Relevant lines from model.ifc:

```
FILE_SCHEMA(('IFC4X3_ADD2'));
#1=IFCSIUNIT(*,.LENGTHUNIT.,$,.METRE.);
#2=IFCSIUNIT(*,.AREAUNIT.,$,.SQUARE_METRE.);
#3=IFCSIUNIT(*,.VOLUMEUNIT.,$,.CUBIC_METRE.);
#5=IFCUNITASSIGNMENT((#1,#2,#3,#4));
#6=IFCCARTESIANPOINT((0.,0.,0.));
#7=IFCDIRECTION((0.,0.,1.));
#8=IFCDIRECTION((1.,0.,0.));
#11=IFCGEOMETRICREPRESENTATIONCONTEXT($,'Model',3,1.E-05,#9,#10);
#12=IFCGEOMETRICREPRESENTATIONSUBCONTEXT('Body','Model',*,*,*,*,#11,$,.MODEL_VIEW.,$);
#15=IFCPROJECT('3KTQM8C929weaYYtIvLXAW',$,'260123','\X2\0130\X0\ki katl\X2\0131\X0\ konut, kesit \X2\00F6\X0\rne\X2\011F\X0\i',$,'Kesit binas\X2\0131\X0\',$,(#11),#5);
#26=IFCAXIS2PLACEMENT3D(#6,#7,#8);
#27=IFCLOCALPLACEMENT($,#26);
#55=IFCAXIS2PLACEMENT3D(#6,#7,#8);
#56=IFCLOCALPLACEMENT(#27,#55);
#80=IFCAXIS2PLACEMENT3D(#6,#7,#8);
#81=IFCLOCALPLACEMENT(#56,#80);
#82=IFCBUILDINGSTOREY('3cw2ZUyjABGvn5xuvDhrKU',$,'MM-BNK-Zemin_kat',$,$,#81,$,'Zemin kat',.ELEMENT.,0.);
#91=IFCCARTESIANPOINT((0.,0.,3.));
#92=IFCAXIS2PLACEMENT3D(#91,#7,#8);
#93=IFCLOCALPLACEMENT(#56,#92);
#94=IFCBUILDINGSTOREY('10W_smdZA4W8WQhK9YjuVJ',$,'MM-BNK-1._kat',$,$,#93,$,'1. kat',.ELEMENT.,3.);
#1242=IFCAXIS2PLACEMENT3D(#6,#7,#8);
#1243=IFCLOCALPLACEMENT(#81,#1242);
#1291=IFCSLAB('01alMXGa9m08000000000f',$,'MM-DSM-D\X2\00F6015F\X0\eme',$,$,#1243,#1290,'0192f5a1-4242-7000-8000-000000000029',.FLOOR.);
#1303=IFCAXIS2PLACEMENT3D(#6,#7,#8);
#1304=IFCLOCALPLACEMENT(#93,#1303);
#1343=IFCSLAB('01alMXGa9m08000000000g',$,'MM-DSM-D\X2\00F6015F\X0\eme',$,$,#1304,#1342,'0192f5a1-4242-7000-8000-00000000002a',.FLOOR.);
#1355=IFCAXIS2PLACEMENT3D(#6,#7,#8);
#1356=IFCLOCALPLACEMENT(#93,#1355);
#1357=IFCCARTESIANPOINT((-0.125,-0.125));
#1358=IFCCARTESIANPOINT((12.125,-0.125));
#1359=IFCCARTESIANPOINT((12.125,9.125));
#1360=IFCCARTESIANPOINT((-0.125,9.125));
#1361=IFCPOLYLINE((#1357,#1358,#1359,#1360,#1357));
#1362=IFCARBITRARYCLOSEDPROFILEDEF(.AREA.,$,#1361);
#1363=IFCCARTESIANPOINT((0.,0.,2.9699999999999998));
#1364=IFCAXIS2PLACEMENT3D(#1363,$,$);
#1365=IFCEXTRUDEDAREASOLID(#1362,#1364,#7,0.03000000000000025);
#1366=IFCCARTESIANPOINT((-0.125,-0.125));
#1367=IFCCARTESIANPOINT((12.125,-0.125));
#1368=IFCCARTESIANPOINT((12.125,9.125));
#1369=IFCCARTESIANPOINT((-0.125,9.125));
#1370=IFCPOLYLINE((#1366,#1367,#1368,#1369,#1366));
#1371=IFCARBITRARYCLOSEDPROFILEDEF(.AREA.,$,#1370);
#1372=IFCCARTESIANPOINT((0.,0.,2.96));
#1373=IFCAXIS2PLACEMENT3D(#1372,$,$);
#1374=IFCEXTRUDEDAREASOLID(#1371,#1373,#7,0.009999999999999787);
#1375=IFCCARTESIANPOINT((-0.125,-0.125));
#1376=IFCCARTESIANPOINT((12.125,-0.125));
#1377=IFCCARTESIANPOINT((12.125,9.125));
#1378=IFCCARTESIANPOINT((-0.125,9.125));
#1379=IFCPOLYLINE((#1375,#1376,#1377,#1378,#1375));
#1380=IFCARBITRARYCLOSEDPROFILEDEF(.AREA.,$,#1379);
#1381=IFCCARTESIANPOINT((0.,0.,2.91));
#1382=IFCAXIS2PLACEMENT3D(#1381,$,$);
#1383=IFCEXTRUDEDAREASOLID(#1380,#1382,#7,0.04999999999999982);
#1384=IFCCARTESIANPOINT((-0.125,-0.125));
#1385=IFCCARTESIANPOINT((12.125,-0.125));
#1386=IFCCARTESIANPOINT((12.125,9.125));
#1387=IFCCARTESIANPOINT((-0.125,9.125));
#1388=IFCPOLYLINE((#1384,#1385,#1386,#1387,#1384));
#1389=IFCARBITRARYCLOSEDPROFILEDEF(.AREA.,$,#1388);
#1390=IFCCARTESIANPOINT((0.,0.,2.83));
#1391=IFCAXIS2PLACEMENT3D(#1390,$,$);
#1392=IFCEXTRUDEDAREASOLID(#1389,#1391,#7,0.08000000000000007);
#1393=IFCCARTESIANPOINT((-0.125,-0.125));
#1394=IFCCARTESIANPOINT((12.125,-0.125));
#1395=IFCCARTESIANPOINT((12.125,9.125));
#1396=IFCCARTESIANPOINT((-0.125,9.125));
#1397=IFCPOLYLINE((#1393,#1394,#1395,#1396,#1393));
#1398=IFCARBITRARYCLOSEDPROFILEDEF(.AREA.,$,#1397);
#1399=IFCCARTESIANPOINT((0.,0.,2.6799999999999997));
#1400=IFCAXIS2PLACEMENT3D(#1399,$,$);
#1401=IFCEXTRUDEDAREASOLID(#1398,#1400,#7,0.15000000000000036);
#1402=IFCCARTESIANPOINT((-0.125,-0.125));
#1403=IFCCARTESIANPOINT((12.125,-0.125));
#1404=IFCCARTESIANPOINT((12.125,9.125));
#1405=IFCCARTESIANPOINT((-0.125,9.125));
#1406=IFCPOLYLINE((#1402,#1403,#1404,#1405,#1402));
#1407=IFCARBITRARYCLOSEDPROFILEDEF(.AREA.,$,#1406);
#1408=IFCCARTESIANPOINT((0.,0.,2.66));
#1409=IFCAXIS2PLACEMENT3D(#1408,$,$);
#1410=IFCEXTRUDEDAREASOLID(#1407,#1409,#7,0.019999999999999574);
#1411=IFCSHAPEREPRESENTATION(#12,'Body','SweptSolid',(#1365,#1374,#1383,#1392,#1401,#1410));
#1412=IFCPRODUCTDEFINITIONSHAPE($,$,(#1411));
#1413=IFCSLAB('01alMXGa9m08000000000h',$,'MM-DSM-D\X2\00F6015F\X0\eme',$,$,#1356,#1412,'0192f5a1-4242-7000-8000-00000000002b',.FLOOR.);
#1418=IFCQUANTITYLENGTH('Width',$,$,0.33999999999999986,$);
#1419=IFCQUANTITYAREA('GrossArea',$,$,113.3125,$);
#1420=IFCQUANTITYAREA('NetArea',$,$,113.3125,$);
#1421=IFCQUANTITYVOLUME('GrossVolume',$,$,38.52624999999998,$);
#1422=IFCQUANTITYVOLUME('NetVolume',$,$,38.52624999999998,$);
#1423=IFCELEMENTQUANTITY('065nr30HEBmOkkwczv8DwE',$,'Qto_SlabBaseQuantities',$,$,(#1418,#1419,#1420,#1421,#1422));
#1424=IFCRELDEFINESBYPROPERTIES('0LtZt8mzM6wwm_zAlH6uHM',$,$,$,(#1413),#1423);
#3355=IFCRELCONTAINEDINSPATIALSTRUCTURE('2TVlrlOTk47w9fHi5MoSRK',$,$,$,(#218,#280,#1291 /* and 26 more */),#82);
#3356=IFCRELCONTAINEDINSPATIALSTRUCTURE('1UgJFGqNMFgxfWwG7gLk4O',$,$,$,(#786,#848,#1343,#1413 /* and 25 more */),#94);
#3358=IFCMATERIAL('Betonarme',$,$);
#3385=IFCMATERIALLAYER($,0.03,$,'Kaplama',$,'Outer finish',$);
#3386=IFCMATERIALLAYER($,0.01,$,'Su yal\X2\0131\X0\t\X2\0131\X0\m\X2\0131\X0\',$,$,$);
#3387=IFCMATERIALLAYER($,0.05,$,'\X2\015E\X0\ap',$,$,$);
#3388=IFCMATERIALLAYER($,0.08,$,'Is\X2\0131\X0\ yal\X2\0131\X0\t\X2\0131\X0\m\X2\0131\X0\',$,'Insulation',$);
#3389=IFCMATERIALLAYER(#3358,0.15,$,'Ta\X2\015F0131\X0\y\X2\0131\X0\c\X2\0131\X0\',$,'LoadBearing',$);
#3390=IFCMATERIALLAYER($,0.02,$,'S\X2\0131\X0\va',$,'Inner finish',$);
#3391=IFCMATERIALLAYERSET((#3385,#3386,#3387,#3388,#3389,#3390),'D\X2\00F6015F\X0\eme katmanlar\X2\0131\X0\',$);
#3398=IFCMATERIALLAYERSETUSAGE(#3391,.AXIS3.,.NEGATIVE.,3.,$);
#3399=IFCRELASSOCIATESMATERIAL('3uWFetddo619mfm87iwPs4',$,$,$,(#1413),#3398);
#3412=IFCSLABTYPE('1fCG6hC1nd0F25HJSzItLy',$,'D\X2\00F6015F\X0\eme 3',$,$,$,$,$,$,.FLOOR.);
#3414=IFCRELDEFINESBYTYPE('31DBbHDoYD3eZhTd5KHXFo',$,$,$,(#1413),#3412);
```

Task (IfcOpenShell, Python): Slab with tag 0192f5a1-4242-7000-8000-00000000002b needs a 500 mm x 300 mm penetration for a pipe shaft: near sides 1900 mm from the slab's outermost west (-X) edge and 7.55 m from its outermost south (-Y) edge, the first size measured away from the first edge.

```python
import numpy as np
import ifcopenshell
import ifcopenshell.api.feature
import ifcopenshell.api.geometry
import ifcopenshell.api.pset
import ifcopenshell.api.root
import ifcopenshell.geom
import ifcopenshell.util.element
import ifcopenshell.util.placement
import ifcopenshell.util.representation
import ifcopenshell.util.shape
import ifcopenshell.util.unit

model = ifcopenshell.open("model.ifc")
unit_scale = ifcopenshell.util.unit.calculate_unit_scale(model)
area_scale = ifcopenshell.util.unit.calculate_unit_scale(model, "AREAUNIT")
volume_scale = ifcopenshell.util.unit.calculate_unit_scale(model, "VOLUMEUNIT")
settings = ifcopenshell.geom.settings()


def volume(element):
    """Net volume in cubic metres, openings subtracted."""
    shape = ifcopenshell.geom.create_shape(settings, element)
    return ifcopenshell.util.shape.get_volume(shape.geometry)


slab = model.by_id(1413)
before = volume(slab)

# Extent in the slab's own axes, in metres. The edges named are its -X and -Y sides.
slab_shape = ifcopenshell.geom.create_shape(settings, slab)
vertices = ifcopenshell.util.shape.get_vertices(slab_shape.geometry)
x_min, y_min, bottom = vertices.min(axis=0)
top = vertices[:, 2].max()

opening = ifcopenshell.api.root.create_entity(model, ifc_class="IfcOpeningElement", name="Pipe shaft opening", predefined_type="OPENING")
context = ifcopenshell.util.representation.get_context(model, "Model", "Body", "MODEL_VIEW")
width, depth = 0.5, 0.3
outline = [(0.0, 0.0), (width, 0.0), (width, depth), (0.0, depth), (0.0, 0.0)]
# Overshoot both faces by 50 mm so the cut is clean.
shape = ifcopenshell.api.geometry.add_slab_representation(
    model, context=context, depth=top - bottom + 0.1, polyline=outline
)
ifcopenshell.api.geometry.assign_representation(model, product=opening, representation=shape)

matrix = ifcopenshell.util.placement.get_local_placement(slab.ObjectPlacement)
matrix[:, 3] = matrix @ np.append(np.array([x_min + 1.9, y_min + 7.55, bottom - 0.05]) / unit_scale, 1.0)
ifcopenshell.api.geometry.edit_object_placement(model, product=opening, matrix=matrix, is_si=False)
ifcopenshell.api.feature.add_feature(model, feature=opening, element=slab)

after = volume(slab)

# Update the slab's stored quantities.
qto = model.by_id(ifcopenshell.util.element.get_pset(slab, "Qto_SlabBaseQuantities", should_inherit=False)["id"])
ifcopenshell.api.pset.edit_qto(model, qto=qto, properties={
    "NetArea": after / (top - bottom) / area_scale,
    "NetVolume": after / volume_scale,
})

print(f"slab volume {before:.3f} -> {after:.3f} m3")

model.write("model_rev.ifc")
```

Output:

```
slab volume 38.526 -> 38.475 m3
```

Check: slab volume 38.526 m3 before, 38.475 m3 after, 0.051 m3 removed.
